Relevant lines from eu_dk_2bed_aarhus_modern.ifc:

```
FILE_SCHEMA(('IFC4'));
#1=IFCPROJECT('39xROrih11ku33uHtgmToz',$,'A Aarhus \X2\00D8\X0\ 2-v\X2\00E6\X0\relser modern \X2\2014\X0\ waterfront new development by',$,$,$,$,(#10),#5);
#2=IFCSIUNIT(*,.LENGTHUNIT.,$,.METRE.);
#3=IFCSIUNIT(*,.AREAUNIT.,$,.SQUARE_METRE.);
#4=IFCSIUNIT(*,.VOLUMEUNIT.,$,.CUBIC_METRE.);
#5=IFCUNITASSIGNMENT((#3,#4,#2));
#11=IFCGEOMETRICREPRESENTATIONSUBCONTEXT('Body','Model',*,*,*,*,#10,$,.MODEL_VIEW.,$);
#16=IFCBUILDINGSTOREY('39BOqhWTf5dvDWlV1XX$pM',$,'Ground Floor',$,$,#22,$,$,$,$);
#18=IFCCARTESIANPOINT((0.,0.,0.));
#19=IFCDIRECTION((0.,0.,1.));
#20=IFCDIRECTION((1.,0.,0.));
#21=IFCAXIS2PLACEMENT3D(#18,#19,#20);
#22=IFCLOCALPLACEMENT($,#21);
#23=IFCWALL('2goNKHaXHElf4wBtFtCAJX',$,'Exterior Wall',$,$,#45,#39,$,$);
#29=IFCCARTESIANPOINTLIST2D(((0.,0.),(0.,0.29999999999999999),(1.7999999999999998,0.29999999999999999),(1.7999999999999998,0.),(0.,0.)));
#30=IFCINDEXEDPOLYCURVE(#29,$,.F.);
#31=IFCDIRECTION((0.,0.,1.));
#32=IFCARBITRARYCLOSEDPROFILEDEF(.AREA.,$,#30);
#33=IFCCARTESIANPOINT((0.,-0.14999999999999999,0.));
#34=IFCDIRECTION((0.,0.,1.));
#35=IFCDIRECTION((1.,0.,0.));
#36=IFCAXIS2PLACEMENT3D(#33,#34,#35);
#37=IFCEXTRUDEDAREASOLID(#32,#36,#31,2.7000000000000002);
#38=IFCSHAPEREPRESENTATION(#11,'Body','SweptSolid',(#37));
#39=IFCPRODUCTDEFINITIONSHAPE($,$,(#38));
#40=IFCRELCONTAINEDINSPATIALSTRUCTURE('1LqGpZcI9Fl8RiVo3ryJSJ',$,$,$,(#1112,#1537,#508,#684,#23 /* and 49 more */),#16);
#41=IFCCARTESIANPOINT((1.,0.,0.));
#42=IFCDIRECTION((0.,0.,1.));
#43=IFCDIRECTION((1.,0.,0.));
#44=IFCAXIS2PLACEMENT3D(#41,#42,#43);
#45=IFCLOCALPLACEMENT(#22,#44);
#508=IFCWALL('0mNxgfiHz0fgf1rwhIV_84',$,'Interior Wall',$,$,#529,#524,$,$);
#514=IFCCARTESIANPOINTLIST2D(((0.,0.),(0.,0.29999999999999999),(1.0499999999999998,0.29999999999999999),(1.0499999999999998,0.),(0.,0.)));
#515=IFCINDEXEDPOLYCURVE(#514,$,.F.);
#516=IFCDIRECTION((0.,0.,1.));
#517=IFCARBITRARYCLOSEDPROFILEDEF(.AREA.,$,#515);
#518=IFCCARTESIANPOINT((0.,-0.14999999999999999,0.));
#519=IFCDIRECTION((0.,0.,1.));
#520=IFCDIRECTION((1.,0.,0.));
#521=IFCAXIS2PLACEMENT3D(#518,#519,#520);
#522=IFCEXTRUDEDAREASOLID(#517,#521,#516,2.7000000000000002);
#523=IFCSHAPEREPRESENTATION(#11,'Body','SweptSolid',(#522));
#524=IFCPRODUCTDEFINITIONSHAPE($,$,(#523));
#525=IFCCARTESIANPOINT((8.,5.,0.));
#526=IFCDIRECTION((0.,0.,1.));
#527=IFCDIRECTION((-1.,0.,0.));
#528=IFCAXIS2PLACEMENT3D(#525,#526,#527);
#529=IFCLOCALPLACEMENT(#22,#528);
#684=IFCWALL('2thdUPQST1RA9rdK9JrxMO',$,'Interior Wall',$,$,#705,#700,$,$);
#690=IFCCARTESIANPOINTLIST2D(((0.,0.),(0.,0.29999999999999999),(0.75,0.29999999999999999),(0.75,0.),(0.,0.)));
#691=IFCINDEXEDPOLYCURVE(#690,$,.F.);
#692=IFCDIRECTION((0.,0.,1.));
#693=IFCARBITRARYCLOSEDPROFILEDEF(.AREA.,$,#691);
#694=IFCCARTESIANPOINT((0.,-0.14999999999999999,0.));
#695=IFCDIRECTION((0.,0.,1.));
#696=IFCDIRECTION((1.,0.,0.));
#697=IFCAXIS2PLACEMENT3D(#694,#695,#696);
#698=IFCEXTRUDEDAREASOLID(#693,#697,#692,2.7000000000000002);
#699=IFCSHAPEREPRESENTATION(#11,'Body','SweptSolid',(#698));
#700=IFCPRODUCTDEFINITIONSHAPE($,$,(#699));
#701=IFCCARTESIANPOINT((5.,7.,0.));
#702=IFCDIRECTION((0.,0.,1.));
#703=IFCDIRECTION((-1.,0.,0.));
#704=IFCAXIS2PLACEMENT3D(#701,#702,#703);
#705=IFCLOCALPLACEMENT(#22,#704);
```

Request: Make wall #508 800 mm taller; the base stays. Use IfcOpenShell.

```python
import ifcopenshell
import ifcopenshell.geom
import ifcopenshell.util.representation
import ifcopenshell.util.shape

model = ifcopenshell.open("eu_dk_2bed_aarhus_modern.ifc")
settings = ifcopenshell.geom.settings()


def volume(element):
    """Net volume in cubic metres, openings subtracted."""
    shape = ifcopenshell.geom.create_shape(settings, element)
    return ifcopenshell.util.shape.get_volume(shape.geometry)


wall = model.by_id(508)
before = volume(wall)

body = ifcopenshell.util.representation.get_representation(wall, "Model", "Body")
solid = body.Items[0]
old_height = solid.Depth
solid.Depth += 0.8
after = volume(wall)

print(f"height {old_height:g} -> {solid.Depth:g}, volume {before:.3f} -> {after:.3f} m3")

model.write("eu_dk_2bed_aarhus_modern_rev.ifc")
```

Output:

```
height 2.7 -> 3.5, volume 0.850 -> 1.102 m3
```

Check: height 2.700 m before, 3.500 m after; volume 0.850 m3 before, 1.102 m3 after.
